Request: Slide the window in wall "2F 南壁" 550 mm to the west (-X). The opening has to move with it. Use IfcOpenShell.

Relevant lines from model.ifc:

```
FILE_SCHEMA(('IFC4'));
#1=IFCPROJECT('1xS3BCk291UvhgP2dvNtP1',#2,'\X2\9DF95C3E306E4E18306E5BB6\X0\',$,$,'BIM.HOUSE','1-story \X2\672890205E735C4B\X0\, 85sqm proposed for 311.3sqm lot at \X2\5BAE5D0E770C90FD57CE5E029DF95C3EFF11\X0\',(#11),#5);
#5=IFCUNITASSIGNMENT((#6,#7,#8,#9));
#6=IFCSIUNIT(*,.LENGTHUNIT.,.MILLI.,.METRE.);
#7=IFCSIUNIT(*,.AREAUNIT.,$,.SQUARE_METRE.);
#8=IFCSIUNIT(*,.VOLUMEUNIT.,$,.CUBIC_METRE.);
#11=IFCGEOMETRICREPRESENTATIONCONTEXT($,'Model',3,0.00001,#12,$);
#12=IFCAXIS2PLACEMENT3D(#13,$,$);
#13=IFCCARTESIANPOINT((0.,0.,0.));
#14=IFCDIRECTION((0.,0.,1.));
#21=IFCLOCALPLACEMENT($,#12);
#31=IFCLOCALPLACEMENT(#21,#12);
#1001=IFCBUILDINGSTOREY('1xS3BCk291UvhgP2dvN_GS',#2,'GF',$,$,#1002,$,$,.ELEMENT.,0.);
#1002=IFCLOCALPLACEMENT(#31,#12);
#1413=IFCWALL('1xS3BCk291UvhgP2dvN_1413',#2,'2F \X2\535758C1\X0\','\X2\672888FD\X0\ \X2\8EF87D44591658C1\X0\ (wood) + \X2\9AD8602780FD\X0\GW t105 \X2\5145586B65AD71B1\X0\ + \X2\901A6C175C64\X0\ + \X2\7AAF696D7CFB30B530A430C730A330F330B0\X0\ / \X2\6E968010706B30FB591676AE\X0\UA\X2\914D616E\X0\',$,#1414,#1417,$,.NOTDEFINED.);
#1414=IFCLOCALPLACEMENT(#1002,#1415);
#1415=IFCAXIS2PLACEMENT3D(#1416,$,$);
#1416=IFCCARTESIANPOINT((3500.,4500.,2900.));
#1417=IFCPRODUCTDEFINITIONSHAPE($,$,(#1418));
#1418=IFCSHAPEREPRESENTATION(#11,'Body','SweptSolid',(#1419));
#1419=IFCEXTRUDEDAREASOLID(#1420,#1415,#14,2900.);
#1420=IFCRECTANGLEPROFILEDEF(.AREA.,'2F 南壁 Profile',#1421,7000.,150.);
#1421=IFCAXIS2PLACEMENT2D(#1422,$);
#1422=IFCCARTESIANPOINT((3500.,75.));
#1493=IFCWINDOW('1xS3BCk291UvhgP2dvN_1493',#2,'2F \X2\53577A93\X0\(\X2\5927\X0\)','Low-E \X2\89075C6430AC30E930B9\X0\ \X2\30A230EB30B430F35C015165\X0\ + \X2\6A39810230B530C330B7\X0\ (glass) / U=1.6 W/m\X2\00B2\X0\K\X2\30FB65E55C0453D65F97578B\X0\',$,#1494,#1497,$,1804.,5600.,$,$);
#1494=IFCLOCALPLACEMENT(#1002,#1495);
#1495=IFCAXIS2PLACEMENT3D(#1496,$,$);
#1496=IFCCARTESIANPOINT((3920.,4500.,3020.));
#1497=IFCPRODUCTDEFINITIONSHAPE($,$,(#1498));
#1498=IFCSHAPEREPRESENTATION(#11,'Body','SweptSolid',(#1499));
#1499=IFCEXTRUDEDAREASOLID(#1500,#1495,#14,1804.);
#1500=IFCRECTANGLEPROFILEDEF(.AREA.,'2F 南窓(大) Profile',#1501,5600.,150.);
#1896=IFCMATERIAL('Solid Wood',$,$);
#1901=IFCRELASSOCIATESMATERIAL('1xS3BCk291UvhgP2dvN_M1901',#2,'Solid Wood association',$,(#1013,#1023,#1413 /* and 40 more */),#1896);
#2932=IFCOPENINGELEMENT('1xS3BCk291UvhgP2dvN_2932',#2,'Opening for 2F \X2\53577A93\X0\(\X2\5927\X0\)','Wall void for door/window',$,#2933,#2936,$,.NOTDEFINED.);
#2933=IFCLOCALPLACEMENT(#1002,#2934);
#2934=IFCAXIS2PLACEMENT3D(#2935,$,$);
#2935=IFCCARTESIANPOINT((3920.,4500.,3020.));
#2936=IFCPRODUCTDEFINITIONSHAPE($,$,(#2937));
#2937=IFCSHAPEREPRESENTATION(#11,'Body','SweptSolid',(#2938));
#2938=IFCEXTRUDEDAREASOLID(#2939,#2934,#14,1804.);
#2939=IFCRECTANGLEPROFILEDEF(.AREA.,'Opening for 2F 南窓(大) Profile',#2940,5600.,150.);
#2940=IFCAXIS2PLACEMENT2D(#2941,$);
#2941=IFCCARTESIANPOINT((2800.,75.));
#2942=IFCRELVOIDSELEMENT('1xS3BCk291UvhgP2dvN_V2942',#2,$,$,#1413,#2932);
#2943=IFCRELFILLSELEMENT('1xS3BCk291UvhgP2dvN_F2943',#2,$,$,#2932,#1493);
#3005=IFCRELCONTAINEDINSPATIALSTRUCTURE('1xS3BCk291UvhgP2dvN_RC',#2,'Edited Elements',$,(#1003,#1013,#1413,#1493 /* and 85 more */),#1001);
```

```python
import ifcopenshell
import ifcopenshell.api.geometry
import ifcopenshell.util.placement

model = ifcopenshell.open("model.ifc")

window = model.by_guid("1xS3BCk291UvhgP2dvN_1493")
opening = window.FillsVoids[0].RelatingOpeningElement
wall = opening.VoidsElements[0].RelatingBuildingElement

wall_matrix = ifcopenshell.util.placement.get_local_placement(wall.ObjectPlacement)
shift = wall_matrix[:3, 0] * -550.0
before = ifcopenshell.util.placement.get_local_placement(window.ObjectPlacement)[:3, 3].copy()

# The window is not placed relative to its opening, so move both.
for product in (opening, window):
    matrix = ifcopenshell.util.placement.get_local_placement(product.ObjectPlacement)
    matrix[:3, 3] += shift
    ifcopenshell.api.geometry.edit_object_placement(model, product=product, matrix=matrix, is_si=False)

after = ifcopenshell.util.placement.get_local_placement(window.ObjectPlacement)[:3, 3]
print("window moved by", (after - before).round(3) + 0.0)

model.write("model_edited.ifc")
```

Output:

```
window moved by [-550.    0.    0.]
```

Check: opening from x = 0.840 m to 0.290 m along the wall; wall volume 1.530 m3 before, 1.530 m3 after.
